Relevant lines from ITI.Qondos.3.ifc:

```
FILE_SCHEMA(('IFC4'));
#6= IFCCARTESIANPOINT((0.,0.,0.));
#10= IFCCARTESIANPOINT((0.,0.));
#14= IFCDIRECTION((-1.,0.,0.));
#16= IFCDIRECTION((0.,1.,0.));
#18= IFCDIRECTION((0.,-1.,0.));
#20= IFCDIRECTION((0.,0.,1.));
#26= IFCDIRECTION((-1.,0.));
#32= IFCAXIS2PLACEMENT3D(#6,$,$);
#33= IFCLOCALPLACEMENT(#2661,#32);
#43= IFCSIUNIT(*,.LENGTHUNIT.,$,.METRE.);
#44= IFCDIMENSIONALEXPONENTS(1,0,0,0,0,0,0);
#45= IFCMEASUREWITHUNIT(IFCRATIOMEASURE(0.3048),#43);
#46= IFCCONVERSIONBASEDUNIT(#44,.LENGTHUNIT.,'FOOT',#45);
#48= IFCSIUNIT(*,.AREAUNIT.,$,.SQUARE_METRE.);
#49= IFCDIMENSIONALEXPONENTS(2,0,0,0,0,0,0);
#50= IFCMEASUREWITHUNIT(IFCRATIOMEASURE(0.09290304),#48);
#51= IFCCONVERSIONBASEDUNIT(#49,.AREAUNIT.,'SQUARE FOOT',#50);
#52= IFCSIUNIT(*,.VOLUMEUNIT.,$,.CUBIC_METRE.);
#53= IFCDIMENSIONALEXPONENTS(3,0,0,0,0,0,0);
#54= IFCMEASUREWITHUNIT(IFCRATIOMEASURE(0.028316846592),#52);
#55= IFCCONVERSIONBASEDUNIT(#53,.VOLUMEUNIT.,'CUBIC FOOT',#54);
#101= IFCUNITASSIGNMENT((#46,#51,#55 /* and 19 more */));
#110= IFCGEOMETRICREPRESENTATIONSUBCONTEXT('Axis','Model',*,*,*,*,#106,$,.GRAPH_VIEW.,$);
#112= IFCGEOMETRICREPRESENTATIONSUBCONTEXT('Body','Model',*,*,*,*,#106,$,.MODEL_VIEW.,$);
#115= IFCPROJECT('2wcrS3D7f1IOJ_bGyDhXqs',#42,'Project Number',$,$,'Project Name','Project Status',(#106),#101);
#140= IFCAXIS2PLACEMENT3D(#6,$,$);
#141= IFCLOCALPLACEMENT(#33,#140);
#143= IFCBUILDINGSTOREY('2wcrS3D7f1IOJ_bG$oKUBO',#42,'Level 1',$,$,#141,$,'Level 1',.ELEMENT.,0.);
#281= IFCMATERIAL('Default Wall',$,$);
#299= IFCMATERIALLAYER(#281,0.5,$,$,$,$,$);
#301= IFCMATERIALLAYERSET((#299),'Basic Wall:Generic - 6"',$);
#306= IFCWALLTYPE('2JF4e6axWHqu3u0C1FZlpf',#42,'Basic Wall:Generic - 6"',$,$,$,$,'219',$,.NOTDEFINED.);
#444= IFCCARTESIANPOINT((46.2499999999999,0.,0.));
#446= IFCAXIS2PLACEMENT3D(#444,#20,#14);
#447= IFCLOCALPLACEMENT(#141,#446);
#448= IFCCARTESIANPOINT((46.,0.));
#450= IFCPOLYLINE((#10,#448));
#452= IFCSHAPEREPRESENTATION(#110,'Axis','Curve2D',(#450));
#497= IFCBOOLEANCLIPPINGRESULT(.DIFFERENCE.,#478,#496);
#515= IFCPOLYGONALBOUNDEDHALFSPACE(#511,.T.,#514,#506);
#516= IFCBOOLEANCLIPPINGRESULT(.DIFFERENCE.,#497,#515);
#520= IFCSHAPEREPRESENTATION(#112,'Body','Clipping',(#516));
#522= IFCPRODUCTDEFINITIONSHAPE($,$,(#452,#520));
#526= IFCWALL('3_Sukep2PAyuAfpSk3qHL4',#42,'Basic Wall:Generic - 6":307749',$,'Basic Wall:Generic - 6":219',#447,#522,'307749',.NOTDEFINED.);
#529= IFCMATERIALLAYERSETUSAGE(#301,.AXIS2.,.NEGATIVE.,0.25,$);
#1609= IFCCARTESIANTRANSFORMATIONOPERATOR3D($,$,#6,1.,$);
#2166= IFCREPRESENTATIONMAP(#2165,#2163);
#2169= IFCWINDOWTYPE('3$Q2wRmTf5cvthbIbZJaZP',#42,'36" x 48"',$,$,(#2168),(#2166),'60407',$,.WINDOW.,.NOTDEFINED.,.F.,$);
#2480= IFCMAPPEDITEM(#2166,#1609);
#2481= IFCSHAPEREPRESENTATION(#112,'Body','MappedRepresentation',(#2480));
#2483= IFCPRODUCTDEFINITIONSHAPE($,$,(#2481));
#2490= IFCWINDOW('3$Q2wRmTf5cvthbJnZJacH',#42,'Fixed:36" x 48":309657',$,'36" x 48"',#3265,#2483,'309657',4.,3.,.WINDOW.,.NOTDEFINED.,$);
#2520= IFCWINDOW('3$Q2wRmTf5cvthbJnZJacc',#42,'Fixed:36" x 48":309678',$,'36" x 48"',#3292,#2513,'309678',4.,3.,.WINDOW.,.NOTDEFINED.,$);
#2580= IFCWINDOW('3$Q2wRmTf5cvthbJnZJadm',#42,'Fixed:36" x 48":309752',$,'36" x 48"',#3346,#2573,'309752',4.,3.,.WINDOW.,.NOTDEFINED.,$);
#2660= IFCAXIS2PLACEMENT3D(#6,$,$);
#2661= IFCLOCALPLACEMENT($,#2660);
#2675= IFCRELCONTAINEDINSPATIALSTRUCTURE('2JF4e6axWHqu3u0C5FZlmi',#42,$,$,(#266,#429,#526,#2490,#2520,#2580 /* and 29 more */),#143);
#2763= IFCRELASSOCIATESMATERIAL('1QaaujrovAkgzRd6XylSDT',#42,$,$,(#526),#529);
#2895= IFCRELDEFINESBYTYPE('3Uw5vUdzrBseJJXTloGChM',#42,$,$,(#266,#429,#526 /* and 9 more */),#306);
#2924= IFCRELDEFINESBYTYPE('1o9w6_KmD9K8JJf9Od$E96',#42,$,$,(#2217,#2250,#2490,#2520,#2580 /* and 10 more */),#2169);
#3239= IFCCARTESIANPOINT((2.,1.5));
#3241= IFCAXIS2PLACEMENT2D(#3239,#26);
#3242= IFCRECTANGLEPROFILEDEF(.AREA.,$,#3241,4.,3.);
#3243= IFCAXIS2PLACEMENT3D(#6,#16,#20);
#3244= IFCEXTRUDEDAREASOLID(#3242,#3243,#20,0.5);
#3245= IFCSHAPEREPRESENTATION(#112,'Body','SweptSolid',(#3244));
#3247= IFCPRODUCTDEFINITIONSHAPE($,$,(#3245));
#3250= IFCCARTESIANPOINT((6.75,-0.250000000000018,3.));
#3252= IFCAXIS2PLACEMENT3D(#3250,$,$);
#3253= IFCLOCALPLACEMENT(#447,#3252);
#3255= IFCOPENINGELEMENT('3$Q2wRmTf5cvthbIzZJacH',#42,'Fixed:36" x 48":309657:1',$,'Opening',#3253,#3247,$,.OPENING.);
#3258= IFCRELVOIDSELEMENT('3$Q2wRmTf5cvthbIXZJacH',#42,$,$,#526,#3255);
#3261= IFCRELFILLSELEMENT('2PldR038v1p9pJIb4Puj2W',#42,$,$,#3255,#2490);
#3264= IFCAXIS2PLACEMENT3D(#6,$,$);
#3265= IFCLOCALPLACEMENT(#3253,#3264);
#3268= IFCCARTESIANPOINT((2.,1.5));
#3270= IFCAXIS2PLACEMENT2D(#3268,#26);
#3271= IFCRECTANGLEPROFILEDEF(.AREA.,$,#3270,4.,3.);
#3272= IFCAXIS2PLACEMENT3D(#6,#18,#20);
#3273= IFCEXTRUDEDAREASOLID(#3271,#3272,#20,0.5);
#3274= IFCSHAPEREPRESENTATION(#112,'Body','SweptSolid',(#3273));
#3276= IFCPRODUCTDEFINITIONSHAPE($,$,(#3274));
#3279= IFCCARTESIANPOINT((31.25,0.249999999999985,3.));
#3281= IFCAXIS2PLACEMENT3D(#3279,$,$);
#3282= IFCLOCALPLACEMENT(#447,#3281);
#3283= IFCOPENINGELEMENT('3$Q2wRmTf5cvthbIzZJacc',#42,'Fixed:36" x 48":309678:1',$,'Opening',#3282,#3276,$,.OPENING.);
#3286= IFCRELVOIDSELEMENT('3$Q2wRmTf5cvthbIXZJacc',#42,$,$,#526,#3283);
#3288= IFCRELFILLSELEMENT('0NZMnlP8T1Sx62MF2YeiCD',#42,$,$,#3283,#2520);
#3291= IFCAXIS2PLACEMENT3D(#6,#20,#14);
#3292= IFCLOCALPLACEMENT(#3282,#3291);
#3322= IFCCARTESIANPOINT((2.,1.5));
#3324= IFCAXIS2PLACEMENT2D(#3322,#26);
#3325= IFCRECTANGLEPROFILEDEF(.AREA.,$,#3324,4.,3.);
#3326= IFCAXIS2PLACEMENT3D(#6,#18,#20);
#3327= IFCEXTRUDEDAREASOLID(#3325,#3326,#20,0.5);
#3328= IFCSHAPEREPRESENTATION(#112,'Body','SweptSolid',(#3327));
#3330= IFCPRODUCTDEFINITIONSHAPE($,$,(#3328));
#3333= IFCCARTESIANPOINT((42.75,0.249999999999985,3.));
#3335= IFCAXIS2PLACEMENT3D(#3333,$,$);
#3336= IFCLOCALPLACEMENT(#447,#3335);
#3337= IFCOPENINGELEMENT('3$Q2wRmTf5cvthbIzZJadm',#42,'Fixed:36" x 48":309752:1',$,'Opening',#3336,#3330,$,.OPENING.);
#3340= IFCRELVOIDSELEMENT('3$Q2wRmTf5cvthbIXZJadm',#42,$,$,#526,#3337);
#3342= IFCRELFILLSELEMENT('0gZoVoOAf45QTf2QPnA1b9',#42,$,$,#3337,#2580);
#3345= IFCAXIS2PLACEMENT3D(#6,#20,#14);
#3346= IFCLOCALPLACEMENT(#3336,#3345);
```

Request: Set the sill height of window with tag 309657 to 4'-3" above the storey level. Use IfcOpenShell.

```python
import numpy as np
import ifcopenshell
import ifcopenshell.api.geometry
import ifcopenshell.geom
import ifcopenshell.util.element
import ifcopenshell.util.placement
import ifcopenshell.util.shape
import ifcopenshell.util.unit

model = ifcopenshell.open("ITI.Qondos.3.ifc")
unit_scale = ifcopenshell.util.unit.calculate_unit_scale(model)

window = model.by_guid("3$Q2wRmTf5cvthbJnZJacH")
opening = window.FillsVoids[0].RelatingOpeningElement
storey = ifcopenshell.util.element.get_container(window, ifc_class="IfcBuildingStorey")
level = ifcopenshell.util.placement.get_local_placement(storey.ObjectPlacement)[2, 3]

# The opening's origin need not be at the sill, so measure its lowest point.
shape = ifcopenshell.geom.create_shape(ifcopenshell.geom.settings(), opening)
bottom = ifcopenshell.util.shape.get_shape_bottom_elevation(shape, shape.geometry) / unit_scale
dz = level + 51 * 0.0254 / unit_scale - bottom

shift = np.array([0.0, 0.0, dz])
# The window is placed relative to its opening, so it follows when the opening moves.
matrix = ifcopenshell.util.placement.get_local_placement(opening.ObjectPlacement)
matrix[:3, 3] += shift
ifcopenshell.api.geometry.edit_object_placement(
    model, product=opening, matrix=matrix, is_si=False, should_transform_children=True
)

print(f"moved by {dz * unit_scale:+.3f} m")

model.write("ITI.Qondos.3_v2.ifc")
```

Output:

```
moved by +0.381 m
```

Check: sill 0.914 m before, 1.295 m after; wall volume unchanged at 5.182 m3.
